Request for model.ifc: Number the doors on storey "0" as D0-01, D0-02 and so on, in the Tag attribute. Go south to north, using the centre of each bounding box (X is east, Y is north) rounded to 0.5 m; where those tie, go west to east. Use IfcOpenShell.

First a look at what the model holds.

```python
import ifcopenshell
import ifcopenshell.util.element
import ifcopenshell.util.placement

model = ifcopenshell.open("model.ifc")
print(model.schema)
storey = next(s for s in model.by_type("IfcBuildingStorey") if s.Name == "0")
doors = [e for e in ifcopenshell.util.element.get_decomposition(storey) if e.is_a("IfcDoor")]
for e in sorted(doors, key=lambda e: e.id()):
    origin = ifcopenshell.util.placement.get_local_placement(e.ObjectPlacement)[:3, 3]
    print(e.id(), e.Tag, e.Name, origin.round(2) + 0.0, sep=" | ")
```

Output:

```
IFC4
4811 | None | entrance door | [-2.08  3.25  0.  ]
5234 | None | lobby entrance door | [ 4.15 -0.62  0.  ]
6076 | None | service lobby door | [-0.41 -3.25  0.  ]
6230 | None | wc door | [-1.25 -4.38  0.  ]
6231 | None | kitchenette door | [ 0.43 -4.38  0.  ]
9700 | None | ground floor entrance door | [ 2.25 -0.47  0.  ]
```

```python
import ifcopenshell
import ifcopenshell.geom
import ifcopenshell.util.element
import ifcopenshell.util.shape

model = ifcopenshell.open("model.ifc")
settings = ifcopenshell.geom.settings()
settings.set("use-world-coords", True)


def centre(element):
    shape = ifcopenshell.geom.create_shape(settings, element)
    return ifcopenshell.util.shape.get_bbox_centroid(shape.geometry)


storey = next(s for s in model.by_type("IfcBuildingStorey") if s.Name == "0")
doors = [e for e in ifcopenshell.util.element.get_decomposition(storey) if e.is_a("IfcDoor")]

# Insertion points can sit at a corner or the storey origin, so sort by the geometry (in metres).
centres = {e: centre(e) for e in doors}
doors.sort(key=lambda e: (round(centres[e][1] / 0.5), centres[e][0]))

for i, e in enumerate(doors, start=1):
    number = f"D0-{i:02d}"
    e.Tag = number
    print(e.id(), number)

model.write("model_rev.ifc")
```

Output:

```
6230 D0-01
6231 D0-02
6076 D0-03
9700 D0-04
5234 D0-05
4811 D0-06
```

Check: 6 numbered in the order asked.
